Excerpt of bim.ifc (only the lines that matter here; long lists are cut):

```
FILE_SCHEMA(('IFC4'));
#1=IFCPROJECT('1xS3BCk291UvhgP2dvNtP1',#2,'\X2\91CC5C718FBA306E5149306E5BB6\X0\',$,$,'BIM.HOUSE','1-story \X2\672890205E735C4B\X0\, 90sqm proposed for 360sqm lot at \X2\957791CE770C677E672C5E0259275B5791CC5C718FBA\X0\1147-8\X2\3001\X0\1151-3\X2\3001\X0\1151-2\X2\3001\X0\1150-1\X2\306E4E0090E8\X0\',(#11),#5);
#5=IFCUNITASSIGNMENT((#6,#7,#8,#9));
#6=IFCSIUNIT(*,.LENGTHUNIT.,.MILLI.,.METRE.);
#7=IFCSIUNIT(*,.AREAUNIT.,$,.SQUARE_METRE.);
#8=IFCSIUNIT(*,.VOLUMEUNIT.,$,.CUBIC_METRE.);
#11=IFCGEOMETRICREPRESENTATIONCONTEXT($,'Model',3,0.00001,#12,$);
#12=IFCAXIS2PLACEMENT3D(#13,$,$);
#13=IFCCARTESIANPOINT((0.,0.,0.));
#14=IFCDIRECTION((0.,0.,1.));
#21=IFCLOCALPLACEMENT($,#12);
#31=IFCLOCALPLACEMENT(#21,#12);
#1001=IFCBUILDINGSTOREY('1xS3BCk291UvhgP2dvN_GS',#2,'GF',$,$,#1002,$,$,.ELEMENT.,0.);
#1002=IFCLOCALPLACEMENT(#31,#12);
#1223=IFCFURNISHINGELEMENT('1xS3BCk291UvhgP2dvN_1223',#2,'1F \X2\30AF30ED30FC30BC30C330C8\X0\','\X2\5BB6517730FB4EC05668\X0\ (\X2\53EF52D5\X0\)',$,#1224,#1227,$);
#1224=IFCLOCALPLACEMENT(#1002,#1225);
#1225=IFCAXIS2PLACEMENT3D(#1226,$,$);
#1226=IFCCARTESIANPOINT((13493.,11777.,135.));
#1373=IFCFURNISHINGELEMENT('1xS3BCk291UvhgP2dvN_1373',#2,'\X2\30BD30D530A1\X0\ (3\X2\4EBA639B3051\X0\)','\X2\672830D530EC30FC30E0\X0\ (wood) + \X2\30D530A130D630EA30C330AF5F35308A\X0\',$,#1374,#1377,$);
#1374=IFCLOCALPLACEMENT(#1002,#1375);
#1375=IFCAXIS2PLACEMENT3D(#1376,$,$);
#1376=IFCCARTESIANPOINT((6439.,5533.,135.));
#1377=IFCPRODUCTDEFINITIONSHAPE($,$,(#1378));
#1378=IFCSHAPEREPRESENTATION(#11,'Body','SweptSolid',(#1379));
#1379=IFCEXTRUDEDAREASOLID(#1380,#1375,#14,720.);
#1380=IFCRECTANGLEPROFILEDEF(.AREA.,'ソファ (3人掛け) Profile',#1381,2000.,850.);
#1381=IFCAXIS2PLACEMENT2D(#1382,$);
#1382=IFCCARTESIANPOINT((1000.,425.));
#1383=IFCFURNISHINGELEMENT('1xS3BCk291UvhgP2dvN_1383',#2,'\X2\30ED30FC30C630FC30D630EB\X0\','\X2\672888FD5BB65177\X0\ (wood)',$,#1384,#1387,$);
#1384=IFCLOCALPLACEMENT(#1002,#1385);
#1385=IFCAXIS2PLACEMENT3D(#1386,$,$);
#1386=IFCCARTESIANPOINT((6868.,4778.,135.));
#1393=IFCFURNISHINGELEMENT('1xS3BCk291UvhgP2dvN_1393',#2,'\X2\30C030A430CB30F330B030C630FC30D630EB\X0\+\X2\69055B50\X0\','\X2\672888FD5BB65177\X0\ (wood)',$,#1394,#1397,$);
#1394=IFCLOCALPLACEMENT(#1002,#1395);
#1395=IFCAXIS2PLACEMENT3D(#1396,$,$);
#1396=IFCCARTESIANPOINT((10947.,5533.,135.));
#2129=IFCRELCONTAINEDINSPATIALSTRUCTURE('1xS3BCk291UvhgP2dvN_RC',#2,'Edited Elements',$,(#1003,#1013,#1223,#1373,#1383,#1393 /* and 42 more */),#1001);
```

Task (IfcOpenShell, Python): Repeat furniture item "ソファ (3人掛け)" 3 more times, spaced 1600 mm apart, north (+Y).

```python
import numpy as np
import ifcopenshell
import ifcopenshell.api.geometry
import ifcopenshell.api.root
import ifcopenshell.util.element
import ifcopenshell.util.placement

model = ifcopenshell.open("bim.ifc")


def reuse_history(source, copy):
    """copy_class also copies each property set's owner history, people and application; keep the originals."""
    for rel in copy.IsDefinedBy:
        if rel.is_a("IfcRelDefinesByProperties") and (history := rel.RelatingPropertyDefinition.OwnerHistory):
            rel.RelatingPropertyDefinition.OwnerHistory = source.OwnerHistory
            ifcopenshell.util.element.remove_deep2(model, history)


source = model.by_id(1373)
base = ifcopenshell.util.placement.get_local_placement(source.ObjectPlacement)
step = np.array([0.0, 1.0, 0.0]) * 1600.0

for i in range(1, 4):
    copy = ifcopenshell.api.root.copy_class(model, product=source)
    copy.Representation = ifcopenshell.util.element.copy_deep(
        model, source.Representation, exclude=["IfcGeometricRepresentationContext", "IfcRepresentationMap"]
    )
    reuse_history(source, copy)
    matrix = base.copy()
    matrix[:3, 3] += i * step
    print("added at", matrix[:3, 3].round(3) + 0.0)
    ifcopenshell.api.geometry.edit_object_placement(model, product=copy, matrix=matrix, is_si=False)

model.write("bim_updated.ifc")
```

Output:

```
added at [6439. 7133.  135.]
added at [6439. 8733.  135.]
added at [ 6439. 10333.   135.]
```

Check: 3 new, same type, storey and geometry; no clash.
